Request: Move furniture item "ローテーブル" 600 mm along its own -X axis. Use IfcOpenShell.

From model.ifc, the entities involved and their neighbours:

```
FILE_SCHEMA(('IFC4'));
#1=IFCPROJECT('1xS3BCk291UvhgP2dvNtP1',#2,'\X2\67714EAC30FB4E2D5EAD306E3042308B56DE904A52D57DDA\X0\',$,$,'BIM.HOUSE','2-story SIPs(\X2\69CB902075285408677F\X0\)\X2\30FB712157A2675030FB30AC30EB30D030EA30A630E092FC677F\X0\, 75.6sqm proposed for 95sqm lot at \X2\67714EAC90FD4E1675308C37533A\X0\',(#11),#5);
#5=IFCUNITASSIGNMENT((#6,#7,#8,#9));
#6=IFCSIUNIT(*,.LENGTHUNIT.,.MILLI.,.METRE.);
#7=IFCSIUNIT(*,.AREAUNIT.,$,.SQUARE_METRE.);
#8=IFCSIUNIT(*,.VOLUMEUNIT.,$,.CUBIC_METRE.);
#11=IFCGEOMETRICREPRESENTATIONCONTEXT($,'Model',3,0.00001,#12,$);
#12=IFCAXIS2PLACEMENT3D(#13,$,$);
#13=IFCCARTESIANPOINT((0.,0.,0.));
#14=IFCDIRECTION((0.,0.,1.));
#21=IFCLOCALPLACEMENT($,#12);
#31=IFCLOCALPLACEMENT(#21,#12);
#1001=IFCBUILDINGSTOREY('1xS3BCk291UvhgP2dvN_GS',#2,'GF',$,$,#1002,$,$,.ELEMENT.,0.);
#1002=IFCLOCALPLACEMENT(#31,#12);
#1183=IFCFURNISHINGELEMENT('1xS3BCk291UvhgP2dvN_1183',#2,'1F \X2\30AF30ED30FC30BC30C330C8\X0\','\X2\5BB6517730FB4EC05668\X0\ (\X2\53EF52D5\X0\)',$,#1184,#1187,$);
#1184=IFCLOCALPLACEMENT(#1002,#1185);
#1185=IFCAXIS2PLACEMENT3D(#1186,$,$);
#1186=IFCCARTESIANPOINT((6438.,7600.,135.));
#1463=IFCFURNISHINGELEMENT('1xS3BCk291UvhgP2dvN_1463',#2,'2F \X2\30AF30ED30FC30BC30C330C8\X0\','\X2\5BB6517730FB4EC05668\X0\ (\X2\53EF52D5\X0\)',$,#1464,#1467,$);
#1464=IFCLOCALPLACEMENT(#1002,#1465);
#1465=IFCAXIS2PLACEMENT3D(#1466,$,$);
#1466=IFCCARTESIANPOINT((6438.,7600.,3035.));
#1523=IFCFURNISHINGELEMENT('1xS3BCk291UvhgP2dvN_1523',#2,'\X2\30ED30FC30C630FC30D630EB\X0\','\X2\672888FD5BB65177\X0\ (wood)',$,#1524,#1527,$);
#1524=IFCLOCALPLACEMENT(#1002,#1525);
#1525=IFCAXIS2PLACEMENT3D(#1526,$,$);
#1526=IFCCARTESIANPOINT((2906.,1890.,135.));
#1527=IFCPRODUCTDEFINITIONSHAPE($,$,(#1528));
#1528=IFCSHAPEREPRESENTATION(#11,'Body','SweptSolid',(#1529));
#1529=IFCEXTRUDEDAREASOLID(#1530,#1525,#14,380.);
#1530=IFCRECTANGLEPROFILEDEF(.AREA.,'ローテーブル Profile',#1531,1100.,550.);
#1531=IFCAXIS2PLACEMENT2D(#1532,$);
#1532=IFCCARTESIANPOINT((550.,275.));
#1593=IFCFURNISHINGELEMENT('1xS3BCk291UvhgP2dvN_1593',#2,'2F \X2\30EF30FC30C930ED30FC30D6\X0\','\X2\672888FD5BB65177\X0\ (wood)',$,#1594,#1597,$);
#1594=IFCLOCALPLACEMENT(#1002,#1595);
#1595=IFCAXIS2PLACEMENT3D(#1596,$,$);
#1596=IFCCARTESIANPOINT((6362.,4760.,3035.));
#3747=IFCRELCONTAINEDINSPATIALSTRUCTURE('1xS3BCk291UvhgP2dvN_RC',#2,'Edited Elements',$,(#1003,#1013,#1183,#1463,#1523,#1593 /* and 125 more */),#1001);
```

```python
import ifcopenshell
import ifcopenshell.api.geometry
import ifcopenshell.util.placement
import ifcopenshell.util.unit

model = ifcopenshell.open("model.ifc")
unit_scale = ifcopenshell.util.unit.calculate_unit_scale(model)

item = model.by_id(1523)
matrix = ifcopenshell.util.placement.get_local_placement(item.ObjectPlacement)
matrix[:3, 3] -= matrix[:3, 0] * 0.6 / unit_scale
ifcopenshell.api.geometry.edit_object_placement(model, product=item, matrix=matrix, is_si=False)

print(ifcopenshell.util.placement.get_local_placement(item.ObjectPlacement).round(3) + 0.0)

model.write("model-out.ifc")
```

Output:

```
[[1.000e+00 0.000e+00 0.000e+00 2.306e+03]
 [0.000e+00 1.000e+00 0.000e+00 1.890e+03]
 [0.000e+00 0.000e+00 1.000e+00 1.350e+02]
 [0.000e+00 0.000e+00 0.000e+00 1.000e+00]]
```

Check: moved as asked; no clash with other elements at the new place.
